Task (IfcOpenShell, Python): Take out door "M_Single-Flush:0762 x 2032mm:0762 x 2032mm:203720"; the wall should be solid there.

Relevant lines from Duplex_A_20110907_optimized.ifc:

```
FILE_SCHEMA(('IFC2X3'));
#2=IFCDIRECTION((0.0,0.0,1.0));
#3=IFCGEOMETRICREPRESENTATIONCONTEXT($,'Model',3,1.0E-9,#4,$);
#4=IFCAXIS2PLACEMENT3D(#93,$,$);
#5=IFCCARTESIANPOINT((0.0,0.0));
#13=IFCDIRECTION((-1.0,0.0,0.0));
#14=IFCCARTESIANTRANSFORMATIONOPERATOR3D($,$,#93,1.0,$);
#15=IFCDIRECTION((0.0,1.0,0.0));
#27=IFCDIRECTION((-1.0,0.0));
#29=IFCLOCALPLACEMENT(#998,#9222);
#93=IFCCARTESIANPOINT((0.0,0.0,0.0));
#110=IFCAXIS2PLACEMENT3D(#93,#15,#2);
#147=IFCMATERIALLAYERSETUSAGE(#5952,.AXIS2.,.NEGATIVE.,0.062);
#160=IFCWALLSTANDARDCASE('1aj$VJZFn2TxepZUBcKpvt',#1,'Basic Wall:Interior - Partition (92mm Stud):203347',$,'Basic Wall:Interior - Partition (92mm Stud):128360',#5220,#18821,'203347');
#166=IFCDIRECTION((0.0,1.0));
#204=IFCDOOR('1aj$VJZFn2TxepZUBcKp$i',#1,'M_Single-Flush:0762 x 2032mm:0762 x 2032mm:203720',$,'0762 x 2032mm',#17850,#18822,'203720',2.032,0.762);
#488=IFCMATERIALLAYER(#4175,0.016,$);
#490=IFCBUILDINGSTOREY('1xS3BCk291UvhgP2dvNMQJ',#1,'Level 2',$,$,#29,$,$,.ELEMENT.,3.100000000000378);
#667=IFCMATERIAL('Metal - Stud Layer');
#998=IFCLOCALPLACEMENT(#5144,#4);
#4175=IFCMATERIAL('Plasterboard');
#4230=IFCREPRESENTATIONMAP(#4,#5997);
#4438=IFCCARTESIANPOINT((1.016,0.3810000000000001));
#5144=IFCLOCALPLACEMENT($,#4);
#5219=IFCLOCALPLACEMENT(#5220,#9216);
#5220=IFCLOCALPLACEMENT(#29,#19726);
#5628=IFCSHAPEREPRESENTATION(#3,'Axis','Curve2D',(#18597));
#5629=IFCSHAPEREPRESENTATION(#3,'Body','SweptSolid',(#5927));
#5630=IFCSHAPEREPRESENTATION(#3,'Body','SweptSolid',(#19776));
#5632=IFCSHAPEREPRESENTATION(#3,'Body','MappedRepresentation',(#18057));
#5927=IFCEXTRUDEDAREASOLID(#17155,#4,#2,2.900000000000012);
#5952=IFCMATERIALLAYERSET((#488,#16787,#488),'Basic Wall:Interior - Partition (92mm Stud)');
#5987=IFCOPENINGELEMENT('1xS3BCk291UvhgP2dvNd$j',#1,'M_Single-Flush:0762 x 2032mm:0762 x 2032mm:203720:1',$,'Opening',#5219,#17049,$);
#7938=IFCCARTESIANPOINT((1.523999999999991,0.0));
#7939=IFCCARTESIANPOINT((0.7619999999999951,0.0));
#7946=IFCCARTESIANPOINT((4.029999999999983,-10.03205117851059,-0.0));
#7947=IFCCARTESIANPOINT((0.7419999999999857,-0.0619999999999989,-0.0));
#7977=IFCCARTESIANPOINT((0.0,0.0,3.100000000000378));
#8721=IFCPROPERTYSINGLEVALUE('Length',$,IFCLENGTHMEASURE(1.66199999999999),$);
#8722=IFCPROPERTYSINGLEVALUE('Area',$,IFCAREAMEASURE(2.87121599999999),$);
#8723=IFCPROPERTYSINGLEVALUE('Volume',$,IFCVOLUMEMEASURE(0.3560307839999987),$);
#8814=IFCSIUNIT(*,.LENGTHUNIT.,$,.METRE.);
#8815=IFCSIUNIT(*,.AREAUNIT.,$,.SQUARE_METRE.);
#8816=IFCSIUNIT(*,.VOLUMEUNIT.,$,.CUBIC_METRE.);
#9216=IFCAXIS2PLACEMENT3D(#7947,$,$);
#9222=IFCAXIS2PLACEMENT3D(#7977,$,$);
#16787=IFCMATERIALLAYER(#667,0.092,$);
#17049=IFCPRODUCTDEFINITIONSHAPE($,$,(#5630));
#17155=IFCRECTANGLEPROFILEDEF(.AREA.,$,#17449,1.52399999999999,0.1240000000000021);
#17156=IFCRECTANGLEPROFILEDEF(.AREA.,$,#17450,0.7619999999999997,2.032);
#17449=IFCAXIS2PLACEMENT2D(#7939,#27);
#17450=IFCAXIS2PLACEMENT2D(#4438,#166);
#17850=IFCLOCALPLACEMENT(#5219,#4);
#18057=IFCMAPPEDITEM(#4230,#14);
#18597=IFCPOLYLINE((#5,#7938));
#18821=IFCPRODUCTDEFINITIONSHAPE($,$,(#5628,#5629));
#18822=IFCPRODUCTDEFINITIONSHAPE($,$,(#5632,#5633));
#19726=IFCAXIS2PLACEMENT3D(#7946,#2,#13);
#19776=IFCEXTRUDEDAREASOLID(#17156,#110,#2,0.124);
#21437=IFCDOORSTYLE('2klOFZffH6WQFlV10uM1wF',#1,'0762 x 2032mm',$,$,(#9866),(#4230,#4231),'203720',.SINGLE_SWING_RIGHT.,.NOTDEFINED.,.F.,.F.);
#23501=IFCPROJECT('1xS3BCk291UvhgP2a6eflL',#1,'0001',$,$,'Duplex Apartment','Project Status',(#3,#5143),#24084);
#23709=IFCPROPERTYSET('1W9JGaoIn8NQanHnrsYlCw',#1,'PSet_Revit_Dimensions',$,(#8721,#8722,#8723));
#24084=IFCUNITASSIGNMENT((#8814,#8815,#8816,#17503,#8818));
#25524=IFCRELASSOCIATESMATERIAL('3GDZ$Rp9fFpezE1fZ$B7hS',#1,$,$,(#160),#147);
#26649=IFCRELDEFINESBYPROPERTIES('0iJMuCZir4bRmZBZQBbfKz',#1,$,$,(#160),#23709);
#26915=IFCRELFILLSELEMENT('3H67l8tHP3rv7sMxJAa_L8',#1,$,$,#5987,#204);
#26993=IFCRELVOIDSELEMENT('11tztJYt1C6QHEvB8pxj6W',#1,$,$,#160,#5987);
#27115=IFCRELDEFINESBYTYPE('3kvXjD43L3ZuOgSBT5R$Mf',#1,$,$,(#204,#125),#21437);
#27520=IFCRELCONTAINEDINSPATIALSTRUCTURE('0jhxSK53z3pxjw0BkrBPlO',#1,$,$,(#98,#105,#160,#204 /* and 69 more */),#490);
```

```python
import ifcopenshell
import ifcopenshell.api.feature
import ifcopenshell.api.pset
import ifcopenshell.api.root
import ifcopenshell.geom
import ifcopenshell.util.element
import ifcopenshell.util.shape
import ifcopenshell.util.unit

model = ifcopenshell.open("Duplex_A_20110907_optimized.ifc")
area_scale = ifcopenshell.util.unit.calculate_unit_scale(model, "AREAUNIT")
volume_scale = ifcopenshell.util.unit.calculate_unit_scale(model, "VOLUMEUNIT")
settings = ifcopenshell.geom.settings()


def volume(element):
    """Net volume in cubic metres, openings subtracted."""
    shape = ifcopenshell.geom.create_shape(settings, element)
    return ifcopenshell.util.shape.get_volume(shape.geometry)


door = model.by_guid("1aj$VJZFn2TxepZUBcKp$i")
opening = door.FillsVoids[0].RelatingOpeningElement
wall = opening.VoidsElements[0].RelatingBuildingElement
before = volume(wall)

ifcopenshell.api.root.remove_product(model, product=door)
ifcopenshell.api.feature.remove_feature(model, feature=opening)

after = volume(wall)
thickness = 0.124  # wall thickness in metres

# Update the wall's stored quantities.
pset = model.by_id(ifcopenshell.util.element.get_pset(wall, "PSet_Revit_Dimensions", should_inherit=False)["id"])
ifcopenshell.api.pset.edit_pset(model, pset=pset, properties={
    "Area": model.create_entity("IfcAreaMeasure", after / thickness / area_scale),
    "Volume": model.create_entity("IfcVolumeMeasure", after / volume_scale),
})

print(f"wall volume {before:.3f} -> {after:.3f} m3")

model.write("Duplex_A_20110907_optimized-out.ifc")
```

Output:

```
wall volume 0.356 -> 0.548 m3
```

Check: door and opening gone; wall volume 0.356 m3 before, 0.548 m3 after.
